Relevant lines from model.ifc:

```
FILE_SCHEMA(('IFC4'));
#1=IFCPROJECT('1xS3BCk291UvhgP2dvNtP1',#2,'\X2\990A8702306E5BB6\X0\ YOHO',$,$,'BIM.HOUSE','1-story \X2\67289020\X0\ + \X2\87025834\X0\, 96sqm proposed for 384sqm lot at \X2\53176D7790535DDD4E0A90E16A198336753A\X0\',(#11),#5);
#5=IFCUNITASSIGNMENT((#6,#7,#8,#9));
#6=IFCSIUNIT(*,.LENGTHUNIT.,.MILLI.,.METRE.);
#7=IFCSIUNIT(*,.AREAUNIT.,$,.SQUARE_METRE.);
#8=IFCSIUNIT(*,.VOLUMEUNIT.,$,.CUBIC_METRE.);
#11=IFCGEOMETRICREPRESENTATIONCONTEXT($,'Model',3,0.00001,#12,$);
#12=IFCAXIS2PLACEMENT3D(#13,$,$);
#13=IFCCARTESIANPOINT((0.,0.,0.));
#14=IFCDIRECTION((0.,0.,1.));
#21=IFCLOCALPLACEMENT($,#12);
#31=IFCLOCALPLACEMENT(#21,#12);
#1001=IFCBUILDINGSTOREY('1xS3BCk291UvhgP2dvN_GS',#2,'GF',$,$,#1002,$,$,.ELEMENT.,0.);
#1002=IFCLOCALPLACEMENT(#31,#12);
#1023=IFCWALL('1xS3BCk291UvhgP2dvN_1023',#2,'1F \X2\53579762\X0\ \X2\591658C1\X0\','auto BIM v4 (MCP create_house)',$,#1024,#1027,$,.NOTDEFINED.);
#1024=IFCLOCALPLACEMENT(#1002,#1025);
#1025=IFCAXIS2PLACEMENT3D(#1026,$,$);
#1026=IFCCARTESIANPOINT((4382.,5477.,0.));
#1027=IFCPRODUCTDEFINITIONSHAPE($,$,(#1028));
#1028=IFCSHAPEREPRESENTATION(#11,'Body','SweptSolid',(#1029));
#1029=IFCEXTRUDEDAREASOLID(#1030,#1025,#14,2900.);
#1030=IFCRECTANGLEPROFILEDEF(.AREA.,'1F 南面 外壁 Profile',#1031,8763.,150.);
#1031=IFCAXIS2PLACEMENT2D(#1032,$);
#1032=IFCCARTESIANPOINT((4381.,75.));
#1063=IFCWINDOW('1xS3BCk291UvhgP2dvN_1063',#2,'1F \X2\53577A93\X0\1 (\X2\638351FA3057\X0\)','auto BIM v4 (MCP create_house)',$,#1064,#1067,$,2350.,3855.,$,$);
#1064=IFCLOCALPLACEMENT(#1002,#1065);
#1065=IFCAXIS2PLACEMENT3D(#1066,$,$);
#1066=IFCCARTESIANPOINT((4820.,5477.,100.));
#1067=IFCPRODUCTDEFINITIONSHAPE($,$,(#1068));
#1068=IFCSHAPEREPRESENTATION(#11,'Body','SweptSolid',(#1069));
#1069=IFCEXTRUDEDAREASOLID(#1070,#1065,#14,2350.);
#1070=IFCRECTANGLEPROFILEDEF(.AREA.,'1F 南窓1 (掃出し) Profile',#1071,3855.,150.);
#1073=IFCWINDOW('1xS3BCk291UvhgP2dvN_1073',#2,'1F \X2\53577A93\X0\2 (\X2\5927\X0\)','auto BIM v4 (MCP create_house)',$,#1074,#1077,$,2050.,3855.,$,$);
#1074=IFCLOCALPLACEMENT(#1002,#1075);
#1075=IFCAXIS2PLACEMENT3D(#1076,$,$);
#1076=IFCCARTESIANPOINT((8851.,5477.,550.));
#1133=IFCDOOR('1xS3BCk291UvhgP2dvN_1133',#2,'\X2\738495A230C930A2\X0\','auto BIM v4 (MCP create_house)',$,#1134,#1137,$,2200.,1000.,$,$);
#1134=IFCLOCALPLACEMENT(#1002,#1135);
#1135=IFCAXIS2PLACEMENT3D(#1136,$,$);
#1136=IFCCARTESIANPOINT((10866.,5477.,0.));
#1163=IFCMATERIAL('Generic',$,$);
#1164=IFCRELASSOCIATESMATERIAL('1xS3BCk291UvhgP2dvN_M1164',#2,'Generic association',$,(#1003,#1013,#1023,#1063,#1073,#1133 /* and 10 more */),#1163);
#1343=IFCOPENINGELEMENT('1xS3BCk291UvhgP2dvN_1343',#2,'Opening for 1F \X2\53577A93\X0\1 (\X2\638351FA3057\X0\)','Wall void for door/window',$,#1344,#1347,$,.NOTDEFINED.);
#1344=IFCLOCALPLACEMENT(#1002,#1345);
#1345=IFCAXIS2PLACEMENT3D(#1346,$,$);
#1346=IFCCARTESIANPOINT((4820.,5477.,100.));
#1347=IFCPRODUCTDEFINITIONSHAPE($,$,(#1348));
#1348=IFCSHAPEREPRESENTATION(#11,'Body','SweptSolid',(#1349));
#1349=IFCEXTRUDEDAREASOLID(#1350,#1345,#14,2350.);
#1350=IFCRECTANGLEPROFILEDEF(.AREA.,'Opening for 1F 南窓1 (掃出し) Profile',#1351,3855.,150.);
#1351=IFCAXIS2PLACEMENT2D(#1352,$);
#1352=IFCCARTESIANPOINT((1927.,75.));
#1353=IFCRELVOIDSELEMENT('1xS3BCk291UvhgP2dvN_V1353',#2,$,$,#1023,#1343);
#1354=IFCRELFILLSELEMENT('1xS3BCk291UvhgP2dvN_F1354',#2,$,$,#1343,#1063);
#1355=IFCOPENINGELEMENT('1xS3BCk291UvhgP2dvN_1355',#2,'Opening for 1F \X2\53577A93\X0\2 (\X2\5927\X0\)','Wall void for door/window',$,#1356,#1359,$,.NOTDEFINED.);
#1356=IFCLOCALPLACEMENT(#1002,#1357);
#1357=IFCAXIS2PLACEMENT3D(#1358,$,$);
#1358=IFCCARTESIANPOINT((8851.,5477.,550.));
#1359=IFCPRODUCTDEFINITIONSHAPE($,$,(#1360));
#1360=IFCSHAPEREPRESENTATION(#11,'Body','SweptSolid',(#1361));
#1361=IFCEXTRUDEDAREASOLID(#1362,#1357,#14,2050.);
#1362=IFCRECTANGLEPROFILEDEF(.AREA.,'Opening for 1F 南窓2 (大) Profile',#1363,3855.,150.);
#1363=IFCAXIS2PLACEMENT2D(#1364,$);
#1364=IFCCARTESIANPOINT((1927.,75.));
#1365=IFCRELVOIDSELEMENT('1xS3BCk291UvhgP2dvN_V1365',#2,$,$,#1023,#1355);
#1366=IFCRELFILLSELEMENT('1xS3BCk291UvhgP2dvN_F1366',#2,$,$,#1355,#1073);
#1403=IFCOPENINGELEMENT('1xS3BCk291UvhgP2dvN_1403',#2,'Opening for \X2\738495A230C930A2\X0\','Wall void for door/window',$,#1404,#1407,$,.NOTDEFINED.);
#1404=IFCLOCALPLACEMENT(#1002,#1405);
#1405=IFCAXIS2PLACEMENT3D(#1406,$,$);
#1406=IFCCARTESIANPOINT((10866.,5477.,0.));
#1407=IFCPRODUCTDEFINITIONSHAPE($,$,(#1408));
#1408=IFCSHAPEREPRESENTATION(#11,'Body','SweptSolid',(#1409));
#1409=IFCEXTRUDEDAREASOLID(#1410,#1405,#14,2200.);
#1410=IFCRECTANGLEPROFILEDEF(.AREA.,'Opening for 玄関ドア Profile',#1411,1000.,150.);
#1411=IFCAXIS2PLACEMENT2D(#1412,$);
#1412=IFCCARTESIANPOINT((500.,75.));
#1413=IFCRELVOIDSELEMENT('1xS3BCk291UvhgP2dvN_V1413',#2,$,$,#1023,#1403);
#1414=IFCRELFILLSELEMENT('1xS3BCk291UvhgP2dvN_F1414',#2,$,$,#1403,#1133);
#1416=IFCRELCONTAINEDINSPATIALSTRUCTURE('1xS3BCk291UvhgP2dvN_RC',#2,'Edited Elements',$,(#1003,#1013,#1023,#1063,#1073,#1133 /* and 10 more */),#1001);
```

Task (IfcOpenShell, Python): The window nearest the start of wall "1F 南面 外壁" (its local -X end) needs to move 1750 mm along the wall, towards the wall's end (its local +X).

```python
import ifcopenshell
import ifcopenshell.api.geometry
import ifcopenshell.util.placement

model = ifcopenshell.open("model.ifc")

window = model.by_id(1063)
opening = window.FillsVoids[0].RelatingOpeningElement
wall = opening.VoidsElements[0].RelatingBuildingElement

wall_matrix = ifcopenshell.util.placement.get_local_placement(wall.ObjectPlacement)
shift = wall_matrix[:3, 0] * 1750.0
before = ifcopenshell.util.placement.get_local_placement(window.ObjectPlacement)[:3, 3].copy()

# The window is not placed relative to its opening, so move both.
for product in (opening, window):
    matrix = ifcopenshell.util.placement.get_local_placement(product.ObjectPlacement)
    matrix[:3, 3] += shift
    ifcopenshell.api.geometry.edit_object_placement(model, product=product, matrix=matrix, is_si=False)

after = ifcopenshell.util.placement.get_local_placement(window.ObjectPlacement)[:3, 3]
print("window moved by", (after - before).round(3) + 0.0)

model.write("model_rev.ifc")
```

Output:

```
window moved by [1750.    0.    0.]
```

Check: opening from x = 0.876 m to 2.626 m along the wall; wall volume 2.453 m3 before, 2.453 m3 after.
